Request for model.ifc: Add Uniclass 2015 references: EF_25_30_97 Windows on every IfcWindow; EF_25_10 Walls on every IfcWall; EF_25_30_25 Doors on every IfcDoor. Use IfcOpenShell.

First a look at what the model holds.

```python
import ifcopenshell

model = ifcopenshell.open("model.ifc")
print(model.schema)
print("classifications:", [c.Name for c in model.by_type("IfcClassification")])
for ifc_class in ("IfcDoor", "IfcRoof", "IfcStair", "IfcWall", "IfcWindow"):
    print(ifc_class, len(model.by_type(ifc_class)))
```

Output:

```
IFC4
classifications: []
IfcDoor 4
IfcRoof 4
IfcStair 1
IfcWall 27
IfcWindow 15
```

```python
import ifcopenshell
import ifcopenshell.api.classification

model = ifcopenshell.open("model.ifc")

system = ifcopenshell.api.classification.add_classification(model, classification="Uniclass 2015")

codes = {
    "IfcWindow": ("EF_25_30_97", "Windows"),
    "IfcWall": ("EF_25_10", "Walls"),
    "IfcDoor": ("EF_25_30_25", "Doors"),
}
for ifc_class, (code, name) in codes.items():
    products = model.by_type(ifc_class)
    ifcopenshell.api.classification.add_reference(
        model, products=products, classification=system, identification=code, name=name
    )
    print(code, len(products))

model.write("model_updated.ifc")
```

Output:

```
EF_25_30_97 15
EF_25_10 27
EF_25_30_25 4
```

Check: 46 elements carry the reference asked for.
